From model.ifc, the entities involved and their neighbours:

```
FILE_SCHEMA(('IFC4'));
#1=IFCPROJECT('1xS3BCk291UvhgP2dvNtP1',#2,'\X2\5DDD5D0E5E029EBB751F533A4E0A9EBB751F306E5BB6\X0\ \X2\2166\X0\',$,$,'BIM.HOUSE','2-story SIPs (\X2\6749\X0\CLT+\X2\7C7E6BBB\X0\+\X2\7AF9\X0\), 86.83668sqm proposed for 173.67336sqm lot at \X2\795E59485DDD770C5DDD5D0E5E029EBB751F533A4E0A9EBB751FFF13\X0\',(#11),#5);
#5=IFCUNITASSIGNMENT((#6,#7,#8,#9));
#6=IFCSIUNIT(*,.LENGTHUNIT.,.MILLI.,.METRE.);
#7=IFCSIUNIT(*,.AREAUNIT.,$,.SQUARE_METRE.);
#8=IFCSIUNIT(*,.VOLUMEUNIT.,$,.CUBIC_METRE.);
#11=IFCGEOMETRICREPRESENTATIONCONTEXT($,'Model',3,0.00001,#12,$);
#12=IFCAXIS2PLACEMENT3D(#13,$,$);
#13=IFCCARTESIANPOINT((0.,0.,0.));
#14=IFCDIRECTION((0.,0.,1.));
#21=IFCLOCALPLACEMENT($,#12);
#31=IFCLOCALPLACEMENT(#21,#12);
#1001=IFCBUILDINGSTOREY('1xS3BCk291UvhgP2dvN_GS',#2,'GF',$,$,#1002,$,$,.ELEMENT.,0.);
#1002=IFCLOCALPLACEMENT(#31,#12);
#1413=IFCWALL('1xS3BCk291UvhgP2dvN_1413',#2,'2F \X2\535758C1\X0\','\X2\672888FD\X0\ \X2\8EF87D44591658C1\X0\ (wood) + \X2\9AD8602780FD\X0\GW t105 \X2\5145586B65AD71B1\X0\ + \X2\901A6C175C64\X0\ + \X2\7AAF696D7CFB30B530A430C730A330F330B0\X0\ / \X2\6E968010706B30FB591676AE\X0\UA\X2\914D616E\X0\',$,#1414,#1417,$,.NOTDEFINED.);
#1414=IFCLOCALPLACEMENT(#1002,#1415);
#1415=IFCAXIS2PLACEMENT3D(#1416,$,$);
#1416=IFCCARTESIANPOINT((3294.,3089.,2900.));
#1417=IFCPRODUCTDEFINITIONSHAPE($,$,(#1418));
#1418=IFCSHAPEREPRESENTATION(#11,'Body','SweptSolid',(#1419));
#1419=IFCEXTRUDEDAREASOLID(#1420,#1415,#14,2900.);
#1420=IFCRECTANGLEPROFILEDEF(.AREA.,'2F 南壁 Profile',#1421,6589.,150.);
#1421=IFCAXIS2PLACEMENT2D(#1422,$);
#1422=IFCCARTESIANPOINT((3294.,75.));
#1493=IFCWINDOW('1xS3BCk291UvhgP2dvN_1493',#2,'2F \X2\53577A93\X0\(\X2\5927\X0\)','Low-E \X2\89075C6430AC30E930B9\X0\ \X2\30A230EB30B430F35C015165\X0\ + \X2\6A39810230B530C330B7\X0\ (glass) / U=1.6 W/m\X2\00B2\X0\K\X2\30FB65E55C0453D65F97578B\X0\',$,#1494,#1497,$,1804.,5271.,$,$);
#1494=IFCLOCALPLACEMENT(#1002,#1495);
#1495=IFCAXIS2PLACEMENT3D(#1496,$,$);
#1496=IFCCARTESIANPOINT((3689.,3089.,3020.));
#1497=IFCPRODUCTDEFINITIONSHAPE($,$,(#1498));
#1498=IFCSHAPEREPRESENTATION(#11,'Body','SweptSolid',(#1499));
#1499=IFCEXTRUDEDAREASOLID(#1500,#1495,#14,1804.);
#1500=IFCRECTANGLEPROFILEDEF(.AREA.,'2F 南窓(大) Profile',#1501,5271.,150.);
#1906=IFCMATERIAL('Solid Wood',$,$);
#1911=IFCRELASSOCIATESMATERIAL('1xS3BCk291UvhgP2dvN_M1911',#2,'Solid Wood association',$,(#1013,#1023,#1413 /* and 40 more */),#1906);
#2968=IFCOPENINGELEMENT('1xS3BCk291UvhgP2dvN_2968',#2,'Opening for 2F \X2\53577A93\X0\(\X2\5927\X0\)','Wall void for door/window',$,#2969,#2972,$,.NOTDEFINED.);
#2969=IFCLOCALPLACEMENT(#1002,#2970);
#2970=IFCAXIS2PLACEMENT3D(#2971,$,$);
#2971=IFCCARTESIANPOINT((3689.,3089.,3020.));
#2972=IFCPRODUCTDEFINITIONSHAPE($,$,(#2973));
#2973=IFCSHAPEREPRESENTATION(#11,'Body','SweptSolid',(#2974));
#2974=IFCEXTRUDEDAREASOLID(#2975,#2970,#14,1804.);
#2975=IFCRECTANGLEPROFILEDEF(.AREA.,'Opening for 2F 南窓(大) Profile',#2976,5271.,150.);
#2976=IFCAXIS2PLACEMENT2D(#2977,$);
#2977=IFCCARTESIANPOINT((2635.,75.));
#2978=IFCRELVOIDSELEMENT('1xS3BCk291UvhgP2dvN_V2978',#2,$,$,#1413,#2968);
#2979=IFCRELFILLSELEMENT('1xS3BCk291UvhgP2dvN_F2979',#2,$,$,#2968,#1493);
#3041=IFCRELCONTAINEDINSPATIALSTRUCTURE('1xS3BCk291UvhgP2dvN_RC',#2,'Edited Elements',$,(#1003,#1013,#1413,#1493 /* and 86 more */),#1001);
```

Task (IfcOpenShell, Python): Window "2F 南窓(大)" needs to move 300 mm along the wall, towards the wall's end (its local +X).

```python
import ifcopenshell
import ifcopenshell.api.geometry
import ifcopenshell.util.placement
import ifcopenshell.util.unit

model = ifcopenshell.open("model.ifc")
unit_scale = ifcopenshell.util.unit.calculate_unit_scale(model)

window = model.by_guid("1xS3BCk291UvhgP2dvN_1493")
opening = window.FillsVoids[0].RelatingOpeningElement
wall = opening.VoidsElements[0].RelatingBuildingElement

wall_matrix = ifcopenshell.util.placement.get_local_placement(wall.ObjectPlacement)
shift = wall_matrix[:3, 0] * 0.3 / unit_scale
before = ifcopenshell.util.placement.get_local_placement(window.ObjectPlacement)[:3, 3].copy()

# The window is not placed relative to its opening, so move both.
for product in (opening, window):
    matrix = ifcopenshell.util.placement.get_local_placement(product.ObjectPlacement)
    matrix[:3, 3] += shift
    ifcopenshell.api.geometry.edit_object_placement(model, product=product, matrix=matrix, is_si=False)

after = ifcopenshell.util.placement.get_local_placement(window.ObjectPlacement)[:3, 3]
print("window moved by", (after - before).round(3) + 0.0)

model.write("model_edited.ifc")
```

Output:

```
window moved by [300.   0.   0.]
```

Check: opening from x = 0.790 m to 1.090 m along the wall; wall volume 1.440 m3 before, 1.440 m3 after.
